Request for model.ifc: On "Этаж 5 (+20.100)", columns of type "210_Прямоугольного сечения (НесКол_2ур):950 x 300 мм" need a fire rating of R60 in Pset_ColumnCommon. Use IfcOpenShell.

First a look at what the model holds.

```python
import ifcopenshell
import ifcopenshell.util.element

model = ifcopenshell.open("model.ifc")
print(model.schema)
storey = next(s for s in model.by_type("IfcBuildingStorey") if s.Name == "Этаж 5 (+20.100)")
columns = [e for e in ifcopenshell.util.element.get_decomposition(storey) if e.is_a("IfcColumn")]
seen = {}
for e in columns:
    element_type = ifcopenshell.util.element.get_type(e)
    key = (element_type.Name if element_type != e and element_type else None, ifcopenshell.util.element.get_pset(e, "Pset_ColumnCommon", "FireRating"))
    seen[key] = seen.get(key, 0) + 1
for (name, value), count in sorted(seen.items(), key=str):
    print(count, "x", name, "|", value)
```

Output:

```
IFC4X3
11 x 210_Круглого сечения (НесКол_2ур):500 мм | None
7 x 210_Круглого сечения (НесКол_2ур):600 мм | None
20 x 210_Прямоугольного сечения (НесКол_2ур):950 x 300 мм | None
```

```python
import ifcopenshell
import ifcopenshell.api.pset
import ifcopenshell.util.element

model = ifcopenshell.open("model.ifc")

storey = next(s for s in model.by_type("IfcBuildingStorey") if s.Name == "Этаж 5 (+20.100)")
columns = [e for e in ifcopenshell.util.element.get_decomposition(storey) if e.is_a("IfcColumn")]

count = 0
for e in columns:
    element_type = ifcopenshell.util.element.get_type(e)
    if element_type in (None, e) or element_type.Name != "210_Прямоугольного сечения (НесКол_2ур):950 x 300 мм":
        continue
    # add_pset returns the element's existing set when there is one.
    pset = ifcopenshell.api.pset.add_pset(model, product=e, name="Pset_ColumnCommon")
    ifcopenshell.api.pset.edit_pset(model, pset=pset, properties={"FireRating": "R60"})
    count += 1

print(count, "columns updated")

model.write("model-out.ifc")
```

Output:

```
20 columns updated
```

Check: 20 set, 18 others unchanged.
